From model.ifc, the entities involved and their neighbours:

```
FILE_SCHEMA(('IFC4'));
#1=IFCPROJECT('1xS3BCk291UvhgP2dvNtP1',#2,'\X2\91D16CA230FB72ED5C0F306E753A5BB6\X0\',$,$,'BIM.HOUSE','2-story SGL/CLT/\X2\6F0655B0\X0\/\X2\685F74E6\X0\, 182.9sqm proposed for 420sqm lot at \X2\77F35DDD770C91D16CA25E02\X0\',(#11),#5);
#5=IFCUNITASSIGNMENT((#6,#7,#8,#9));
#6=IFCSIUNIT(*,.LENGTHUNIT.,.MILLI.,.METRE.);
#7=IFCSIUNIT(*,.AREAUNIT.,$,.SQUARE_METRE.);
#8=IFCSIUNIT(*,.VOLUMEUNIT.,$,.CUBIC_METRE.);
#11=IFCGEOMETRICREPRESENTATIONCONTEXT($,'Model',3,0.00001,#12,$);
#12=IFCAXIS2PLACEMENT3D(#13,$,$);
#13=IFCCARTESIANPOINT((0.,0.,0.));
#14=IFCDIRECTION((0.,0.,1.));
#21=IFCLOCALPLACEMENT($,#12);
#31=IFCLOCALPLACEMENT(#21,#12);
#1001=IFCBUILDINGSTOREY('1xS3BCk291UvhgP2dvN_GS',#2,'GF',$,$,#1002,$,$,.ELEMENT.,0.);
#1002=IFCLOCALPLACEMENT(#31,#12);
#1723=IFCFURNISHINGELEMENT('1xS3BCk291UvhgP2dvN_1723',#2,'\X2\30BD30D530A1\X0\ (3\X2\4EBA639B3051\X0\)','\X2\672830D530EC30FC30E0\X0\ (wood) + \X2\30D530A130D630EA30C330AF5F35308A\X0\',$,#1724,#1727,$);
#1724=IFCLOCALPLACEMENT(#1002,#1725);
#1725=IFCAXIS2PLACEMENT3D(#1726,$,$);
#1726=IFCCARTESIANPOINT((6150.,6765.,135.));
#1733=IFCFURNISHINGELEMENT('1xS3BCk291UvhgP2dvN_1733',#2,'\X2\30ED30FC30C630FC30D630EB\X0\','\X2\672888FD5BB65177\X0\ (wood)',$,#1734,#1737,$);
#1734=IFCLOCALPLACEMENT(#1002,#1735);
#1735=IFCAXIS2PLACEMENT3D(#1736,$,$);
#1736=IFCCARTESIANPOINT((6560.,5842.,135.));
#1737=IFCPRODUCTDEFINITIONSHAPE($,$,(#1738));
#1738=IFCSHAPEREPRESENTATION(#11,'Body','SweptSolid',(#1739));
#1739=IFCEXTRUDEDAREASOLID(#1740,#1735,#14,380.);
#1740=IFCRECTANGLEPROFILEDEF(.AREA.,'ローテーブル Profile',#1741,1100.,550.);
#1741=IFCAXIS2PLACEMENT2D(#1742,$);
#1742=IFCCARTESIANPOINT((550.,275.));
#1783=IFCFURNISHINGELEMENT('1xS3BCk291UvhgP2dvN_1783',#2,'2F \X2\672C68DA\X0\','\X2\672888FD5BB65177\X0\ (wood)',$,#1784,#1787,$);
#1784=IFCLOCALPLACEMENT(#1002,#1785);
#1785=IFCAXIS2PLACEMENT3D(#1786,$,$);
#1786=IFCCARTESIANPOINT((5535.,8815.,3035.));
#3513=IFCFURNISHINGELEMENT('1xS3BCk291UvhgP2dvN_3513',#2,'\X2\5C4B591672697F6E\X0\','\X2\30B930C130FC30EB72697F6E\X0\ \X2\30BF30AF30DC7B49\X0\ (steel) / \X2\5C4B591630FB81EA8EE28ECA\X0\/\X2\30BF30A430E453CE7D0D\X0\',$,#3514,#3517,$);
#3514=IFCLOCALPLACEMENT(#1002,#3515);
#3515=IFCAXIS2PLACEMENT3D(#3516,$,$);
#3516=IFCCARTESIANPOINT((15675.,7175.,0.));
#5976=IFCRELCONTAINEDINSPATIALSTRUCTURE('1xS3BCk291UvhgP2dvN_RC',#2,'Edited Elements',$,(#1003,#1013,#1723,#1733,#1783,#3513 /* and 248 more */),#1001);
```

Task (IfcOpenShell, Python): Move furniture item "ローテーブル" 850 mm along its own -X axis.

```python
import ifcopenshell
import ifcopenshell.api.geometry
import ifcopenshell.util.placement
import ifcopenshell.util.unit

model = ifcopenshell.open("model.ifc")
unit_scale = ifcopenshell.util.unit.calculate_unit_scale(model)

item = model.by_guid("1xS3BCk291UvhgP2dvN_1733")
matrix = ifcopenshell.util.placement.get_local_placement(item.ObjectPlacement)
matrix[:3, 3] -= matrix[:3, 0] * 0.85 / unit_scale
ifcopenshell.api.geometry.edit_object_placement(model, product=item, matrix=matrix, is_si=False)

print(ifcopenshell.util.placement.get_local_placement(item.ObjectPlacement).round(3) + 0.0)

model.write("model_v2.ifc")
```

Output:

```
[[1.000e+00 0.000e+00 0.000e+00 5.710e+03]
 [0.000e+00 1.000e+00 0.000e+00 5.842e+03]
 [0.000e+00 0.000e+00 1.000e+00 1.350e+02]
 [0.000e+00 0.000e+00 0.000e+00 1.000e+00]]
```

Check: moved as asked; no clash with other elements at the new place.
